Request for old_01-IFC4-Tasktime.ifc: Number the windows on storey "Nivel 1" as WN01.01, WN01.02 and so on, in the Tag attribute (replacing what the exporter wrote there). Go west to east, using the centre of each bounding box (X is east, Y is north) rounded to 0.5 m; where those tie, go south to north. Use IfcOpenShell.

First a look at what the model holds.

```python
import ifcopenshell
import ifcopenshell.util.element
import ifcopenshell.util.placement

model = ifcopenshell.open("old_01-IFC4-Tasktime.ifc")
print(model.schema)
storey = next(s for s in model.by_type("IfcBuildingStorey") if s.Name == "Nivel 1")
windows = [e for e in ifcopenshell.util.element.get_decomposition(storey) if e.is_a("IfcWindow")]
for e in sorted(windows, key=lambda e: e.id()):
    origin = ifcopenshell.util.placement.get_local_placement(e.ObjectPlacement)[:3, 3]
    print(e.id(), e.Tag, e.Name, origin.round(2) + 0.0, sep=" | ")
```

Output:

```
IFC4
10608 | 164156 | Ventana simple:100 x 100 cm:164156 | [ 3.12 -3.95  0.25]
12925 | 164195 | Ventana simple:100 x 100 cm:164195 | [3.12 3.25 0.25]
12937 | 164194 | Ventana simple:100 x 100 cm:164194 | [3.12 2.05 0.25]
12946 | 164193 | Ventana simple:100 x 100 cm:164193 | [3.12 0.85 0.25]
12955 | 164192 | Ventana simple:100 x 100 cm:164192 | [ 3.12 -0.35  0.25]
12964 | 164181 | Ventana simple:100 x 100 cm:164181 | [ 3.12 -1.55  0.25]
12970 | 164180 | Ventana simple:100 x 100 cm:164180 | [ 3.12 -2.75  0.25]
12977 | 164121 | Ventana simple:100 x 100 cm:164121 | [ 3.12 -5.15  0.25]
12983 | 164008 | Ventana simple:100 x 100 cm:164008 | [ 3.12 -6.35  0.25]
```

```python
import ifcopenshell
import ifcopenshell.geom
import ifcopenshell.util.element
import ifcopenshell.util.shape

model = ifcopenshell.open("old_01-IFC4-Tasktime.ifc")
settings = ifcopenshell.geom.settings()
settings.set("use-world-coords", True)


def centre(element):
    shape = ifcopenshell.geom.create_shape(settings, element)
    return ifcopenshell.util.shape.get_bbox_centroid(shape.geometry)


storey = next(s for s in model.by_type("IfcBuildingStorey") if s.Name == "Nivel 1")
windows = [e for e in ifcopenshell.util.element.get_decomposition(storey) if e.is_a("IfcWindow")]

# Insertion points can sit at a corner or the storey origin, so sort by the geometry (in metres).
centres = {e: centre(e) for e in windows}
windows.sort(key=lambda e: (round(centres[e][0] / 0.5), centres[e][1]))

for i, e in enumerate(windows, start=1):
    number = f"WN01.{i:02d}"
    e.Tag = number
    print(e.id(), number)

model.write("old_01-IFC4-Tasktime_v2.ifc")
```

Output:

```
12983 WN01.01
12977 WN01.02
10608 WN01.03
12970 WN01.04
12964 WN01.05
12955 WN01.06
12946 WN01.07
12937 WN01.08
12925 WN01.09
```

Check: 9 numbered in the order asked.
